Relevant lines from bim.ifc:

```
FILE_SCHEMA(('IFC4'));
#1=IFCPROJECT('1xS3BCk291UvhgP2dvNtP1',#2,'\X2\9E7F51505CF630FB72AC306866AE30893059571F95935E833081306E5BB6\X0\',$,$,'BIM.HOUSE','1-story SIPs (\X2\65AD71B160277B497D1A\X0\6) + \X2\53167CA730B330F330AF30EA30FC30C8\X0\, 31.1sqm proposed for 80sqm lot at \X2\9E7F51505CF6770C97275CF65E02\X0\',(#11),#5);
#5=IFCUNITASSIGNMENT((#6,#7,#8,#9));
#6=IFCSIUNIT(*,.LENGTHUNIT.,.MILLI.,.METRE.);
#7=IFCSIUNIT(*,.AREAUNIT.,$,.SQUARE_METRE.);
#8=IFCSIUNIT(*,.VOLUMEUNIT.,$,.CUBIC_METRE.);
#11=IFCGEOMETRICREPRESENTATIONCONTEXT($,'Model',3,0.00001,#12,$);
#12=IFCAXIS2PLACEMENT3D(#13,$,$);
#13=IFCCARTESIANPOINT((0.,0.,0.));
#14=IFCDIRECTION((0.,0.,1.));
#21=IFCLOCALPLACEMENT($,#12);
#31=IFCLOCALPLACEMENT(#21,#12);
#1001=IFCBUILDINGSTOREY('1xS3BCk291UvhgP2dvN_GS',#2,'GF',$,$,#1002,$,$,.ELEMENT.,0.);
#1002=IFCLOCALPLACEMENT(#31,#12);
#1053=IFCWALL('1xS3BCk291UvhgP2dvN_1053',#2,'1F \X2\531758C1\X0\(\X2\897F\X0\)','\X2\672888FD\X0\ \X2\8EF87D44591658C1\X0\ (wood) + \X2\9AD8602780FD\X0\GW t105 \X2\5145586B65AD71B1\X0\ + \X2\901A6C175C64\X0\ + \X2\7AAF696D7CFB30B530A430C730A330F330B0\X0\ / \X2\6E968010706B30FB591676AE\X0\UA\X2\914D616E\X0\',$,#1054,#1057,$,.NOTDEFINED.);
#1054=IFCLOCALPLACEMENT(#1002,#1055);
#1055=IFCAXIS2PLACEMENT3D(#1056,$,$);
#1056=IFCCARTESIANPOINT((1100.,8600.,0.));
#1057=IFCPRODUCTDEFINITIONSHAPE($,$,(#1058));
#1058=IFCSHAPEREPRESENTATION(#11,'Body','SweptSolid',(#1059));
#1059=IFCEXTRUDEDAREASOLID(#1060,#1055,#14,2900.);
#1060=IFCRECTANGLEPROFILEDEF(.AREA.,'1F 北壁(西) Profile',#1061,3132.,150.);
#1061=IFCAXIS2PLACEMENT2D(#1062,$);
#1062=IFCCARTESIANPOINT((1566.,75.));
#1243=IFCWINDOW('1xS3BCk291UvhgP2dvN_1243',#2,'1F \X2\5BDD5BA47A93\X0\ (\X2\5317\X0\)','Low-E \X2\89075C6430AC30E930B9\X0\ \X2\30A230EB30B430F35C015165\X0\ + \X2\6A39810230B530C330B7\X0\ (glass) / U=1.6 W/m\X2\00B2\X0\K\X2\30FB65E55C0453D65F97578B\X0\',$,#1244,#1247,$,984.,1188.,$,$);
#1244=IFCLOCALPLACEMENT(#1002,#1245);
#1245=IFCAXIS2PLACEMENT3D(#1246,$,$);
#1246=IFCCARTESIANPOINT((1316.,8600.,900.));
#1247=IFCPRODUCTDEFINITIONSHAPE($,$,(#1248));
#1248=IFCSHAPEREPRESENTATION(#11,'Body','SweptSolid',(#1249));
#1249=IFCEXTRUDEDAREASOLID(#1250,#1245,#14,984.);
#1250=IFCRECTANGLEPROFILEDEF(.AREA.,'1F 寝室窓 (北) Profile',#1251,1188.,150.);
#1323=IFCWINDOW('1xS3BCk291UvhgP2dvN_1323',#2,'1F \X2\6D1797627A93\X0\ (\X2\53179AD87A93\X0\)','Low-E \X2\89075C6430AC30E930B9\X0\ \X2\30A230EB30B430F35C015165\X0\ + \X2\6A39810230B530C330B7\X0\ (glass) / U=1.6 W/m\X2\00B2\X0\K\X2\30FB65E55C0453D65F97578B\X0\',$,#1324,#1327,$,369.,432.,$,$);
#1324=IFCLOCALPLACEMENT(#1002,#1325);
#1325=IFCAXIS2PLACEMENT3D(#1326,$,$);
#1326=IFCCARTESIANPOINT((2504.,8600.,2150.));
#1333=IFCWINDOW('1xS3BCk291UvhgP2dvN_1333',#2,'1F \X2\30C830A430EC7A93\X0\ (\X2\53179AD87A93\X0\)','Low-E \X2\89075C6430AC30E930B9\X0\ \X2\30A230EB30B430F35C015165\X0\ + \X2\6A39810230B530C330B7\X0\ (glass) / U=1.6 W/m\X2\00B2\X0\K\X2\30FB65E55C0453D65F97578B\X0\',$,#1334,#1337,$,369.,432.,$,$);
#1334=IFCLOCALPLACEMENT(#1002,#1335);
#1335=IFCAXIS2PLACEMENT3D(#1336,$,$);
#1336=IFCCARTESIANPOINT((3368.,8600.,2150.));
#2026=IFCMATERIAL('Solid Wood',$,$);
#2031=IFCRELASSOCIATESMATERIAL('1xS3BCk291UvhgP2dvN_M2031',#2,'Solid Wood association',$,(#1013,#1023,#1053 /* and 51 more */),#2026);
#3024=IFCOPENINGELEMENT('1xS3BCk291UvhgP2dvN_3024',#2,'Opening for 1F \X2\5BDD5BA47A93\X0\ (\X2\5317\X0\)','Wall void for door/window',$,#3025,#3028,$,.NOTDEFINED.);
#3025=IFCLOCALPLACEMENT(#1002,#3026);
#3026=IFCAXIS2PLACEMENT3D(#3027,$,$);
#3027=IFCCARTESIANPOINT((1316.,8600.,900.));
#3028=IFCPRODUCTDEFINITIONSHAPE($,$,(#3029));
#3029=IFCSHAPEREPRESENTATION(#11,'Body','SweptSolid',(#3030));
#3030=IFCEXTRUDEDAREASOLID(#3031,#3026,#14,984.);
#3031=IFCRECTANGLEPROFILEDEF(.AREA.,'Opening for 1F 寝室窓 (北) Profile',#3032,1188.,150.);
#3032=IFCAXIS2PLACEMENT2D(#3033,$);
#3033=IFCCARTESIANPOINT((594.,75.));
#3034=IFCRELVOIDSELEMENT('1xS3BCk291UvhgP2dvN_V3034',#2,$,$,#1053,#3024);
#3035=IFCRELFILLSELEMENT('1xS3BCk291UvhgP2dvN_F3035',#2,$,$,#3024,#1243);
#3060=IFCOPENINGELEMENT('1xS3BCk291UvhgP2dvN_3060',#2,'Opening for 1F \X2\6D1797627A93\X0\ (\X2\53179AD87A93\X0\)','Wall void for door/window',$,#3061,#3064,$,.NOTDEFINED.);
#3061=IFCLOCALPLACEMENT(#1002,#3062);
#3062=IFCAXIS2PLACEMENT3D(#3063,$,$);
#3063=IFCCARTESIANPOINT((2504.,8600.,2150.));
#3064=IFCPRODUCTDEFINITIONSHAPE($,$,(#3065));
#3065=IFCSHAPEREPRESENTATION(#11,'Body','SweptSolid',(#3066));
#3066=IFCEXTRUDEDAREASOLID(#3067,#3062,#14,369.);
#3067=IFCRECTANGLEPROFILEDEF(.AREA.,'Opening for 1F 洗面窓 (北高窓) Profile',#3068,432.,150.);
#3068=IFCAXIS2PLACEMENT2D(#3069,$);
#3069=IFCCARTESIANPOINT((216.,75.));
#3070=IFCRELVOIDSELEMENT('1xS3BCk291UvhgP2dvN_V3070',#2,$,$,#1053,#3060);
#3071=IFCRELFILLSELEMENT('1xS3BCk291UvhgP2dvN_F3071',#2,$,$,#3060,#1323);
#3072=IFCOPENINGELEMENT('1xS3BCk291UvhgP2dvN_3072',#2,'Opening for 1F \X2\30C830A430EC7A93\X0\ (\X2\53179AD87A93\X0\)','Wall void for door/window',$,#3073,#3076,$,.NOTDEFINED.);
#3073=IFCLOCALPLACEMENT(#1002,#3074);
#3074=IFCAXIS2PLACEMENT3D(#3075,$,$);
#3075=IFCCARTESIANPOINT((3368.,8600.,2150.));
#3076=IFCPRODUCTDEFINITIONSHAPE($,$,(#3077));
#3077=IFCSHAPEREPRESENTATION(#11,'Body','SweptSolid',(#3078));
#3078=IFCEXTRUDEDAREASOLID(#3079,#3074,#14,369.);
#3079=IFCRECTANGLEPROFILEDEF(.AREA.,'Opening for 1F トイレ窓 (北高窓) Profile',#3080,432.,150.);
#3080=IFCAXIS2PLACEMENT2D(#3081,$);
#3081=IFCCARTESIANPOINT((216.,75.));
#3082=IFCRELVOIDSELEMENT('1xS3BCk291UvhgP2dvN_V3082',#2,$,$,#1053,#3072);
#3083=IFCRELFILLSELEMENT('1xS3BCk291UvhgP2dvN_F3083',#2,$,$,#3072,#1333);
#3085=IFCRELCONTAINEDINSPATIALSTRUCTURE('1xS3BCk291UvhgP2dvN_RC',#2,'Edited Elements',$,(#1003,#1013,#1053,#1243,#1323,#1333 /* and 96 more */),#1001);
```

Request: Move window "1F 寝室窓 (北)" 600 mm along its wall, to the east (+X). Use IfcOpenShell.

```python
import ifcopenshell
import ifcopenshell.api.geometry
import ifcopenshell.util.placement

model = ifcopenshell.open("bim.ifc")

window = model.by_guid("1xS3BCk291UvhgP2dvN_1243")
opening = window.FillsVoids[0].RelatingOpeningElement
wall = opening.VoidsElements[0].RelatingBuildingElement

wall_matrix = ifcopenshell.util.placement.get_local_placement(wall.ObjectPlacement)
shift = wall_matrix[:3, 0] * 600.0
before = ifcopenshell.util.placement.get_local_placement(window.ObjectPlacement)[:3, 3].copy()

# The window is not placed relative to its opening, so move both.
for product in (opening, window):
    matrix = ifcopenshell.util.placement.get_local_placement(product.ObjectPlacement)
    matrix[:3, 3] += shift
    ifcopenshell.api.geometry.edit_object_placement(model, product=product, matrix=matrix, is_si=False)

after = ifcopenshell.util.placement.get_local_placement(window.ObjectPlacement)[:3, 3]
print("window moved by", (after - before).round(3) + 0.0)

model.write("bim_edited.ifc")
```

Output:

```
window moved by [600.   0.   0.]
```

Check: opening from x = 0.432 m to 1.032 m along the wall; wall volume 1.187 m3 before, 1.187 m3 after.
